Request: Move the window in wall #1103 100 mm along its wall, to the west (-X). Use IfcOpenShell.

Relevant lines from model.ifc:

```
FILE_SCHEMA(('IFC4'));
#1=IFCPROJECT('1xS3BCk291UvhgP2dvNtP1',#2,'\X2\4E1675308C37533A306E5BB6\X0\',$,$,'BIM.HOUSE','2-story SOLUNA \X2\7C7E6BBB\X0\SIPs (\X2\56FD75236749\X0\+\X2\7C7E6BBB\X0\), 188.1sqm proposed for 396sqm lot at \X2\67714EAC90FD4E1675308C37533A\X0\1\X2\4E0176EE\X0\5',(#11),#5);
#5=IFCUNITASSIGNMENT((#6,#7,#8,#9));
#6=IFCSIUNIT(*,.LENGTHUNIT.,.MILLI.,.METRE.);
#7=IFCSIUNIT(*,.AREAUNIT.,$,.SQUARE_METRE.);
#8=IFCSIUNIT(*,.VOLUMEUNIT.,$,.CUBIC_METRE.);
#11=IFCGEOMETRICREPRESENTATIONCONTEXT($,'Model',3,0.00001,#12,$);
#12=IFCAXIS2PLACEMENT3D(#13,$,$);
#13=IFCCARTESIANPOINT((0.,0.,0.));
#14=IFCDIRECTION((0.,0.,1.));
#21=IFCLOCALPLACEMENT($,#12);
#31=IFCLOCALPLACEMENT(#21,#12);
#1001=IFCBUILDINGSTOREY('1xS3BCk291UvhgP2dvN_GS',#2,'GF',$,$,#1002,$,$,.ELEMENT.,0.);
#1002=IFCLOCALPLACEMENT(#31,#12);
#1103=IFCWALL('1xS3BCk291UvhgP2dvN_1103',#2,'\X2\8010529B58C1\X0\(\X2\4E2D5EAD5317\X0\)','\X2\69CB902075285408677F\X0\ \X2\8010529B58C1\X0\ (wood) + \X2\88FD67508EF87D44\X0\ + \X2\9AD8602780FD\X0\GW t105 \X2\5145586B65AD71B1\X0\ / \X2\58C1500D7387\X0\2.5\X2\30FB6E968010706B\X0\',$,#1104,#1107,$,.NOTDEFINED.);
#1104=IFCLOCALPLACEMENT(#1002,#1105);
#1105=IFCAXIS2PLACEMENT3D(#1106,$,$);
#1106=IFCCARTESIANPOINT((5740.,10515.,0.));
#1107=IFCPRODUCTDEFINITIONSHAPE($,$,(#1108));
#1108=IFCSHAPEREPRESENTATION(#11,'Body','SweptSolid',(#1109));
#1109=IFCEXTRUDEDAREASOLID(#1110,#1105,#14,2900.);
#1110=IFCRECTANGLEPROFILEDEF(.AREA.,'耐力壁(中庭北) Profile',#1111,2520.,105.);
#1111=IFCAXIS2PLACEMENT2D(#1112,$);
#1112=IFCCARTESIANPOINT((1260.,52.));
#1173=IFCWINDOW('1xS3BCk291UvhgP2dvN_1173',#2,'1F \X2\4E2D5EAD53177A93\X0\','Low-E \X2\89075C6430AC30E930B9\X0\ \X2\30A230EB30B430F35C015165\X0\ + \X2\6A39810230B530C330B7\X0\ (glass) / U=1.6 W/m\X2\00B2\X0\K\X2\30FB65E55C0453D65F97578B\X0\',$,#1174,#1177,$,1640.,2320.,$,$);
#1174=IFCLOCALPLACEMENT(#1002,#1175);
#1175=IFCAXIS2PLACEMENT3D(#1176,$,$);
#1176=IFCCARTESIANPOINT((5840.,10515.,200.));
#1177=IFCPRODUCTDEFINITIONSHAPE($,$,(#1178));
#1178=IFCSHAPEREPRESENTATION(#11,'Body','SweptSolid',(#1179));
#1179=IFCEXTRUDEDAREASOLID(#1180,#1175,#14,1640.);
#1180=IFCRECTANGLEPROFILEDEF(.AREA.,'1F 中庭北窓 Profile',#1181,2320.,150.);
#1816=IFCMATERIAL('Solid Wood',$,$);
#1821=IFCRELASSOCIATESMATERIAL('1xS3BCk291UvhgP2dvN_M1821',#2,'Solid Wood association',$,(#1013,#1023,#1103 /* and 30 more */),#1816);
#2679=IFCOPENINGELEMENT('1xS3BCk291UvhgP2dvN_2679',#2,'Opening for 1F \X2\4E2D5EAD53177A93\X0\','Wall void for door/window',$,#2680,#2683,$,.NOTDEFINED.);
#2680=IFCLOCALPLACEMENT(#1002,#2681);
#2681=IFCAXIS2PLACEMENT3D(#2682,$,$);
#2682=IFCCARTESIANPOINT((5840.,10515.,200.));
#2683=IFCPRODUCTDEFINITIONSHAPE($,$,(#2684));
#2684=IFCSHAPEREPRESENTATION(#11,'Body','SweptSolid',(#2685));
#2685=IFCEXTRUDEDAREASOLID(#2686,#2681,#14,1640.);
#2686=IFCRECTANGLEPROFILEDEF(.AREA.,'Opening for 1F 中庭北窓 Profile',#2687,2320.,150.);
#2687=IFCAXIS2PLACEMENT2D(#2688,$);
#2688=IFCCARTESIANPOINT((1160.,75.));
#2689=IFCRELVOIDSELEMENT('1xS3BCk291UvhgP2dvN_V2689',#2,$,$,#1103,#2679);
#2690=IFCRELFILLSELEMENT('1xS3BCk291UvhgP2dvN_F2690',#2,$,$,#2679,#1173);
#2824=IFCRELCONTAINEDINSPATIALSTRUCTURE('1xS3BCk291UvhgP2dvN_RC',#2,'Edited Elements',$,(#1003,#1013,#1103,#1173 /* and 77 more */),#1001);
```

```python
import ifcopenshell
import ifcopenshell.api.geometry
import ifcopenshell.util.placement
import ifcopenshell.util.unit

model = ifcopenshell.open("model.ifc")
unit_scale = ifcopenshell.util.unit.calculate_unit_scale(model)

window = model.by_guid("1xS3BCk291UvhgP2dvN_1173")
opening = window.FillsVoids[0].RelatingOpeningElement
wall = opening.VoidsElements[0].RelatingBuildingElement

wall_matrix = ifcopenshell.util.placement.get_local_placement(wall.ObjectPlacement)
shift = wall_matrix[:3, 0] * -0.1 / unit_scale
before = ifcopenshell.util.placement.get_local_placement(window.ObjectPlacement)[:3, 3].copy()

# The window is not placed relative to its opening, so move both.
for product in (opening, window):
    matrix = ifcopenshell.util.placement.get_local_placement(product.ObjectPlacement)
    matrix[:3, 3] += shift
    ifcopenshell.api.geometry.edit_object_placement(model, product=product, matrix=matrix, is_si=False)

after = ifcopenshell.util.placement.get_local_placement(window.ObjectPlacement)[:3, 3]
print("window moved by", (after - before).round(3) + 0.0)

model.write("model-out.ifc")
```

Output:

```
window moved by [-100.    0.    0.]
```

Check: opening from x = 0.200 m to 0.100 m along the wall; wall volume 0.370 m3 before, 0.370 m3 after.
